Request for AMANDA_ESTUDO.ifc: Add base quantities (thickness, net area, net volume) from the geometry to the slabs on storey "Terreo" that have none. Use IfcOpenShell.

First a look at what the model holds.

```python
import ifcopenshell
import ifcopenshell.util.element
import ifcopenshell.util.unit

model = ifcopenshell.open("AMANDA_ESTUDO.ifc")
print(model.schema)
for unit_type in ("LENGTHUNIT", "AREAUNIT", "VOLUMEUNIT"):
    print(unit_type, ifcopenshell.util.unit.calculate_unit_scale(model, unit_type))
storey = next(s for s in model.by_type("IfcBuildingStorey") if s.Name == "Terreo")
slabs = [e for e in ifcopenshell.util.element.get_decomposition(storey) if e.is_a("IfcSlab")]
for e in sorted(slabs, key=lambda e: e.id()):
    print(e.id(), e.is_a(), e.Name, list(ifcopenshell.util.element.get_psets(e, qtos_only=True)), sep=" | ")
```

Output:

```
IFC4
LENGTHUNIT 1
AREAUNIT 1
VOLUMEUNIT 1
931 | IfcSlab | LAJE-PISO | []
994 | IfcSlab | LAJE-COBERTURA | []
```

```python
import ifcopenshell
import ifcopenshell.api.pset
import ifcopenshell.geom
import ifcopenshell.util.element
import ifcopenshell.util.shape
import ifcopenshell.util.unit

model = ifcopenshell.open("AMANDA_ESTUDO.ifc")
unit_scale = ifcopenshell.util.unit.calculate_unit_scale(model)
area_scale = ifcopenshell.util.unit.calculate_unit_scale(model, "AREAUNIT")
volume_scale = ifcopenshell.util.unit.calculate_unit_scale(model, "VOLUMEUNIT")
settings = ifcopenshell.geom.settings()

storey = next(s for s in model.by_type("IfcBuildingStorey") if s.Name == "Terreo")
slabs = [e for e in ifcopenshell.util.element.get_decomposition(storey) if e.is_a("IfcSlab")]

for e in sorted(slabs, key=lambda e: e.id()):
    if ifcopenshell.util.element.get_psets(e, qtos_only=True, should_inherit=False):
        continue
    # Geometry comes back in metres, in the element's own axes.
    shape = ifcopenshell.geom.create_shape(settings, e)
    values = {
        "Width": ifcopenshell.util.shape.get_z(shape.geometry) / unit_scale,
        "NetArea": ifcopenshell.util.shape.get_footprint_area(shape.geometry) / area_scale,
        "NetVolume": ifcopenshell.util.shape.get_volume(shape.geometry) / volume_scale,
    }
    qto = ifcopenshell.api.pset.add_qto(model, product=e, name="Qto_SlabBaseQuantities")
    ifcopenshell.api.pset.edit_qto(model, qto=qto, properties=values)
    print(e.id(), {k: round(v, 3) for k, v in values.items()})

model.write("AMANDA_ESTUDO-out.ifc")
```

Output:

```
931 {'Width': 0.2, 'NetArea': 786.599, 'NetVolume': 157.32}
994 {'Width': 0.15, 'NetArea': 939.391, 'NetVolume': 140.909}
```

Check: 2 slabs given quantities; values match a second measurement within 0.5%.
